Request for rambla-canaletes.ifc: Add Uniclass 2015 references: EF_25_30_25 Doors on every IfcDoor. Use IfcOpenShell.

First a look at what the model holds.

```python
import ifcopenshell

model = ifcopenshell.open("rambla-canaletes.ifc")
print(model.schema)
print("classifications:", [c.Name for c in model.by_type("IfcClassification")])
for ifc_class in ("IfcDoor", "IfcRoof", "IfcStair", "IfcWall", "IfcWindow"):
    print(ifc_class, len(model.by_type(ifc_class)))
```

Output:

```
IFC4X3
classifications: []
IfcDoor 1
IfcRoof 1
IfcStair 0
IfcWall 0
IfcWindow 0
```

```python
import ifcopenshell
import ifcopenshell.api.classification

model = ifcopenshell.open("rambla-canaletes.ifc")

system = ifcopenshell.api.classification.add_classification(model, classification="Uniclass 2015")

codes = {
    "IfcDoor": ("EF_25_30_25", "Doors"),
}
for ifc_class, (code, name) in codes.items():
    products = model.by_type(ifc_class)
    ifcopenshell.api.classification.add_reference(
        model, products=products, classification=system, identification=code, name=name
    )
    print(code, len(products))

model.write("rambla-canaletes-out.ifc")
```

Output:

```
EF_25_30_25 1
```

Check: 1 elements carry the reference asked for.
